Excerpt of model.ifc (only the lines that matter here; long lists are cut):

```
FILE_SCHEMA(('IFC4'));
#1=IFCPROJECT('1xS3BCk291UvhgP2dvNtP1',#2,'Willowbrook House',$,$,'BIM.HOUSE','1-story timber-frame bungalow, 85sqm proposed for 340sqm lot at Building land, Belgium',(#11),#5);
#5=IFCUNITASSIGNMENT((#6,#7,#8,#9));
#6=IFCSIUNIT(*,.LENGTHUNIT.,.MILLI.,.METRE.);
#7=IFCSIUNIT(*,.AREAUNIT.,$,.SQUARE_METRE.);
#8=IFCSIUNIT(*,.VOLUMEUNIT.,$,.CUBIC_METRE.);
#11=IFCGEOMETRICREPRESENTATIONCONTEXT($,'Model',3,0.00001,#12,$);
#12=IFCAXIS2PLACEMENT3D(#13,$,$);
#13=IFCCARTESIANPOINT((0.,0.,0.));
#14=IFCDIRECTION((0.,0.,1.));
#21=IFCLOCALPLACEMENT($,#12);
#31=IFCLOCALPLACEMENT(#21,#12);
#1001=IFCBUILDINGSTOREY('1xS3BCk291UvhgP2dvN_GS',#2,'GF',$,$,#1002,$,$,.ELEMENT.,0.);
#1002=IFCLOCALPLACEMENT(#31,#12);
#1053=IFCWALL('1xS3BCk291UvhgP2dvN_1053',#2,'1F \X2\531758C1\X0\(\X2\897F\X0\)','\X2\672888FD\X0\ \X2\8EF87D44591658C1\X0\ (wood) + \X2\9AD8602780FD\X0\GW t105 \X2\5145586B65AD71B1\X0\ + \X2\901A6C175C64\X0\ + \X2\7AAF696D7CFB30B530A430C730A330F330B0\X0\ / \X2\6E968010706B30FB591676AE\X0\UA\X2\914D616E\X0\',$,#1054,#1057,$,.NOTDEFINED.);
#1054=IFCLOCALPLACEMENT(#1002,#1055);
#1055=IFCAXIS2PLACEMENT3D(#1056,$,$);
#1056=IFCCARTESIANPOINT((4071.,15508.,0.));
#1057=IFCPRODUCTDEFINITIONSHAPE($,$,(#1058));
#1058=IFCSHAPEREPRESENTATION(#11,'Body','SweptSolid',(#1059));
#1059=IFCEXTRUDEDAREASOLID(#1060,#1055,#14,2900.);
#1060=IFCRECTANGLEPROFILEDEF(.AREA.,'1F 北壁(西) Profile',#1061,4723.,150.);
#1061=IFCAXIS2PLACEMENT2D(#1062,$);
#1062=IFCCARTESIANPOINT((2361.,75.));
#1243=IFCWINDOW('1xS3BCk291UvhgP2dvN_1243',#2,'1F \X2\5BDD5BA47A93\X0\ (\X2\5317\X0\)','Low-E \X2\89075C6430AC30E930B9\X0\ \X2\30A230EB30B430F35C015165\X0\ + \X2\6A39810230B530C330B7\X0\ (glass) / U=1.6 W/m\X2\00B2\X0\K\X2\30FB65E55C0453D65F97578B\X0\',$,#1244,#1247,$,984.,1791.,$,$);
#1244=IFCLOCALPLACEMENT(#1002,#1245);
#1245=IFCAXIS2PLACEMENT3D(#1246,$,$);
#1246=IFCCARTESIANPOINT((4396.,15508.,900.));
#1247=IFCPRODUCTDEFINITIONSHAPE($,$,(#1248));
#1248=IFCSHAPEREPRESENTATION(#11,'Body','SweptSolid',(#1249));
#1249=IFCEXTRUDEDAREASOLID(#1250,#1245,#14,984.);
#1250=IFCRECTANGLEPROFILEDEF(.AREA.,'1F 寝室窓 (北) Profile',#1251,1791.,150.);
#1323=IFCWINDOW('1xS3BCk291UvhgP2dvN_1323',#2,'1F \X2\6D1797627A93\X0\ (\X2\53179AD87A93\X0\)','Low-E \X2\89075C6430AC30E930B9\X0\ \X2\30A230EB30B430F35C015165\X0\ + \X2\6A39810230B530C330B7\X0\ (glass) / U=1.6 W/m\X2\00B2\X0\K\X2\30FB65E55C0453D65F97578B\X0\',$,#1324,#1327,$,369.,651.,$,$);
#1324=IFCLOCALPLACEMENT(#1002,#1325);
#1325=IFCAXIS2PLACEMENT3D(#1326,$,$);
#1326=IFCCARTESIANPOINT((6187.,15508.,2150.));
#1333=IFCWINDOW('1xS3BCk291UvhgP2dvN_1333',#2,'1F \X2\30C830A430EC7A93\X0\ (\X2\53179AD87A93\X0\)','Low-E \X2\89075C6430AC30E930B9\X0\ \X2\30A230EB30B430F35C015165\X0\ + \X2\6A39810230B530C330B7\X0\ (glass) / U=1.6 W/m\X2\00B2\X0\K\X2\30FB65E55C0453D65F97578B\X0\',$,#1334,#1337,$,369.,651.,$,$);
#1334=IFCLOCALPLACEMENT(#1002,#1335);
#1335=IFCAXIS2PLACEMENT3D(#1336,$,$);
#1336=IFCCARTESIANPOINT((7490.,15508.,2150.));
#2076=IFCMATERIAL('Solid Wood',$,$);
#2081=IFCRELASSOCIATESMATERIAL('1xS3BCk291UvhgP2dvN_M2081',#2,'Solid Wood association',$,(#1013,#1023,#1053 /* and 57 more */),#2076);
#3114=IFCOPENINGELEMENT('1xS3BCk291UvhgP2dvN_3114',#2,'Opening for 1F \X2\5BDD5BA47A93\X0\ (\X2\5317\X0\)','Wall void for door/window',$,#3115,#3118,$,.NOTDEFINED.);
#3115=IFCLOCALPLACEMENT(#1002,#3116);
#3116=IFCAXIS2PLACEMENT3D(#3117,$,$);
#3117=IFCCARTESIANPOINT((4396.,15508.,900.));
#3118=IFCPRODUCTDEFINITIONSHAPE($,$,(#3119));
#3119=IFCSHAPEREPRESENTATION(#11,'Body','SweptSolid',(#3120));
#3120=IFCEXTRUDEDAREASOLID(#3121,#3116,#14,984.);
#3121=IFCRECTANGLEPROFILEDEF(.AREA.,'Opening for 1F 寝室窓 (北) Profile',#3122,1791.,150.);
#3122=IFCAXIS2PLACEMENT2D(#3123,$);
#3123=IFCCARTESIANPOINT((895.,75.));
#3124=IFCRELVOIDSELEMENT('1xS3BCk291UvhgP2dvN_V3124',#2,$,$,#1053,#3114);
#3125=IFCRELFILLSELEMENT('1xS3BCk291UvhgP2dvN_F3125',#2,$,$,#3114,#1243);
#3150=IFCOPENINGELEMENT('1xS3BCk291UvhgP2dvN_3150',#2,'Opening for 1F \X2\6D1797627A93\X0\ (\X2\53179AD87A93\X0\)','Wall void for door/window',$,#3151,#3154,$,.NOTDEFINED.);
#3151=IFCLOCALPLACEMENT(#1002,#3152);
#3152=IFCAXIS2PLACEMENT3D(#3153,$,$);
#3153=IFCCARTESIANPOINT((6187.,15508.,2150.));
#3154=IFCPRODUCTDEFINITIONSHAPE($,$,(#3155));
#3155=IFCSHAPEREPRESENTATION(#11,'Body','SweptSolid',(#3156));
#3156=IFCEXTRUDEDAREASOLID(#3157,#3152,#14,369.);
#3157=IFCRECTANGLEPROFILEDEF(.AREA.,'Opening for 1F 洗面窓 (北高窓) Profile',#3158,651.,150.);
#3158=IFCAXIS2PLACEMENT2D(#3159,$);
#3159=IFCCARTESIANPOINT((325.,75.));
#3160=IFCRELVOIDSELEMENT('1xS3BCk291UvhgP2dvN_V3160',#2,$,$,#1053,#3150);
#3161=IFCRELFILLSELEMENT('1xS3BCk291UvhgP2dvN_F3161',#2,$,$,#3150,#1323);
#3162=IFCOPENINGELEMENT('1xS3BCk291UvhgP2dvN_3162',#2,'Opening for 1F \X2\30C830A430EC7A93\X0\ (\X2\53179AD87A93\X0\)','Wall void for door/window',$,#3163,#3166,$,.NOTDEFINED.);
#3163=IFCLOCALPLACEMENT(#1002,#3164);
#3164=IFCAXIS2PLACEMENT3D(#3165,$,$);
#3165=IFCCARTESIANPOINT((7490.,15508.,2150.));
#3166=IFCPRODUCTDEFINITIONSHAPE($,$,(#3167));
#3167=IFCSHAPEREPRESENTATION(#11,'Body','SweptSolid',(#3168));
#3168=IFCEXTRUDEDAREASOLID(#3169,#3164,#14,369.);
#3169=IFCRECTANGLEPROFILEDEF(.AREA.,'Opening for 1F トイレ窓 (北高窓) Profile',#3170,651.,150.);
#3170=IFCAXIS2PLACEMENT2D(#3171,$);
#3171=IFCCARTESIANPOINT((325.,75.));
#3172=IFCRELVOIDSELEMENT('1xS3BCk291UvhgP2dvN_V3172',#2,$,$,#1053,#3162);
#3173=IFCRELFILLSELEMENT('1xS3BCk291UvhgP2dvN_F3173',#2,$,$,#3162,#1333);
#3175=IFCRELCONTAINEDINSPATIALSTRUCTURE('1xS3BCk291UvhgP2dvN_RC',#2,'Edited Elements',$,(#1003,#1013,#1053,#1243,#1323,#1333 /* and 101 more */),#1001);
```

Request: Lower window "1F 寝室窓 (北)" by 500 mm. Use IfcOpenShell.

```python
import numpy as np
import ifcopenshell
import ifcopenshell.api.geometry
import ifcopenshell.util.placement
import ifcopenshell.util.unit

model = ifcopenshell.open("model.ifc")
unit_scale = ifcopenshell.util.unit.calculate_unit_scale(model)

window = model.by_guid("1xS3BCk291UvhgP2dvN_1243")
opening = window.FillsVoids[0].RelatingOpeningElement
dz = -0.5 / unit_scale

shift = np.array([0.0, 0.0, dz])
# The window is not placed relative to its opening, so move both.
for product in (opening, window):
    matrix = ifcopenshell.util.placement.get_local_placement(product.ObjectPlacement)
    matrix[:3, 3] += shift
    ifcopenshell.api.geometry.edit_object_placement(model, product=product, matrix=matrix, is_si=False)

print(f"moved by {dz * unit_scale:+.3f} m")

model.write("model_updated.ifc")
```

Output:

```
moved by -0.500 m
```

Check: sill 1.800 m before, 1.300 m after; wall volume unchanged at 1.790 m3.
